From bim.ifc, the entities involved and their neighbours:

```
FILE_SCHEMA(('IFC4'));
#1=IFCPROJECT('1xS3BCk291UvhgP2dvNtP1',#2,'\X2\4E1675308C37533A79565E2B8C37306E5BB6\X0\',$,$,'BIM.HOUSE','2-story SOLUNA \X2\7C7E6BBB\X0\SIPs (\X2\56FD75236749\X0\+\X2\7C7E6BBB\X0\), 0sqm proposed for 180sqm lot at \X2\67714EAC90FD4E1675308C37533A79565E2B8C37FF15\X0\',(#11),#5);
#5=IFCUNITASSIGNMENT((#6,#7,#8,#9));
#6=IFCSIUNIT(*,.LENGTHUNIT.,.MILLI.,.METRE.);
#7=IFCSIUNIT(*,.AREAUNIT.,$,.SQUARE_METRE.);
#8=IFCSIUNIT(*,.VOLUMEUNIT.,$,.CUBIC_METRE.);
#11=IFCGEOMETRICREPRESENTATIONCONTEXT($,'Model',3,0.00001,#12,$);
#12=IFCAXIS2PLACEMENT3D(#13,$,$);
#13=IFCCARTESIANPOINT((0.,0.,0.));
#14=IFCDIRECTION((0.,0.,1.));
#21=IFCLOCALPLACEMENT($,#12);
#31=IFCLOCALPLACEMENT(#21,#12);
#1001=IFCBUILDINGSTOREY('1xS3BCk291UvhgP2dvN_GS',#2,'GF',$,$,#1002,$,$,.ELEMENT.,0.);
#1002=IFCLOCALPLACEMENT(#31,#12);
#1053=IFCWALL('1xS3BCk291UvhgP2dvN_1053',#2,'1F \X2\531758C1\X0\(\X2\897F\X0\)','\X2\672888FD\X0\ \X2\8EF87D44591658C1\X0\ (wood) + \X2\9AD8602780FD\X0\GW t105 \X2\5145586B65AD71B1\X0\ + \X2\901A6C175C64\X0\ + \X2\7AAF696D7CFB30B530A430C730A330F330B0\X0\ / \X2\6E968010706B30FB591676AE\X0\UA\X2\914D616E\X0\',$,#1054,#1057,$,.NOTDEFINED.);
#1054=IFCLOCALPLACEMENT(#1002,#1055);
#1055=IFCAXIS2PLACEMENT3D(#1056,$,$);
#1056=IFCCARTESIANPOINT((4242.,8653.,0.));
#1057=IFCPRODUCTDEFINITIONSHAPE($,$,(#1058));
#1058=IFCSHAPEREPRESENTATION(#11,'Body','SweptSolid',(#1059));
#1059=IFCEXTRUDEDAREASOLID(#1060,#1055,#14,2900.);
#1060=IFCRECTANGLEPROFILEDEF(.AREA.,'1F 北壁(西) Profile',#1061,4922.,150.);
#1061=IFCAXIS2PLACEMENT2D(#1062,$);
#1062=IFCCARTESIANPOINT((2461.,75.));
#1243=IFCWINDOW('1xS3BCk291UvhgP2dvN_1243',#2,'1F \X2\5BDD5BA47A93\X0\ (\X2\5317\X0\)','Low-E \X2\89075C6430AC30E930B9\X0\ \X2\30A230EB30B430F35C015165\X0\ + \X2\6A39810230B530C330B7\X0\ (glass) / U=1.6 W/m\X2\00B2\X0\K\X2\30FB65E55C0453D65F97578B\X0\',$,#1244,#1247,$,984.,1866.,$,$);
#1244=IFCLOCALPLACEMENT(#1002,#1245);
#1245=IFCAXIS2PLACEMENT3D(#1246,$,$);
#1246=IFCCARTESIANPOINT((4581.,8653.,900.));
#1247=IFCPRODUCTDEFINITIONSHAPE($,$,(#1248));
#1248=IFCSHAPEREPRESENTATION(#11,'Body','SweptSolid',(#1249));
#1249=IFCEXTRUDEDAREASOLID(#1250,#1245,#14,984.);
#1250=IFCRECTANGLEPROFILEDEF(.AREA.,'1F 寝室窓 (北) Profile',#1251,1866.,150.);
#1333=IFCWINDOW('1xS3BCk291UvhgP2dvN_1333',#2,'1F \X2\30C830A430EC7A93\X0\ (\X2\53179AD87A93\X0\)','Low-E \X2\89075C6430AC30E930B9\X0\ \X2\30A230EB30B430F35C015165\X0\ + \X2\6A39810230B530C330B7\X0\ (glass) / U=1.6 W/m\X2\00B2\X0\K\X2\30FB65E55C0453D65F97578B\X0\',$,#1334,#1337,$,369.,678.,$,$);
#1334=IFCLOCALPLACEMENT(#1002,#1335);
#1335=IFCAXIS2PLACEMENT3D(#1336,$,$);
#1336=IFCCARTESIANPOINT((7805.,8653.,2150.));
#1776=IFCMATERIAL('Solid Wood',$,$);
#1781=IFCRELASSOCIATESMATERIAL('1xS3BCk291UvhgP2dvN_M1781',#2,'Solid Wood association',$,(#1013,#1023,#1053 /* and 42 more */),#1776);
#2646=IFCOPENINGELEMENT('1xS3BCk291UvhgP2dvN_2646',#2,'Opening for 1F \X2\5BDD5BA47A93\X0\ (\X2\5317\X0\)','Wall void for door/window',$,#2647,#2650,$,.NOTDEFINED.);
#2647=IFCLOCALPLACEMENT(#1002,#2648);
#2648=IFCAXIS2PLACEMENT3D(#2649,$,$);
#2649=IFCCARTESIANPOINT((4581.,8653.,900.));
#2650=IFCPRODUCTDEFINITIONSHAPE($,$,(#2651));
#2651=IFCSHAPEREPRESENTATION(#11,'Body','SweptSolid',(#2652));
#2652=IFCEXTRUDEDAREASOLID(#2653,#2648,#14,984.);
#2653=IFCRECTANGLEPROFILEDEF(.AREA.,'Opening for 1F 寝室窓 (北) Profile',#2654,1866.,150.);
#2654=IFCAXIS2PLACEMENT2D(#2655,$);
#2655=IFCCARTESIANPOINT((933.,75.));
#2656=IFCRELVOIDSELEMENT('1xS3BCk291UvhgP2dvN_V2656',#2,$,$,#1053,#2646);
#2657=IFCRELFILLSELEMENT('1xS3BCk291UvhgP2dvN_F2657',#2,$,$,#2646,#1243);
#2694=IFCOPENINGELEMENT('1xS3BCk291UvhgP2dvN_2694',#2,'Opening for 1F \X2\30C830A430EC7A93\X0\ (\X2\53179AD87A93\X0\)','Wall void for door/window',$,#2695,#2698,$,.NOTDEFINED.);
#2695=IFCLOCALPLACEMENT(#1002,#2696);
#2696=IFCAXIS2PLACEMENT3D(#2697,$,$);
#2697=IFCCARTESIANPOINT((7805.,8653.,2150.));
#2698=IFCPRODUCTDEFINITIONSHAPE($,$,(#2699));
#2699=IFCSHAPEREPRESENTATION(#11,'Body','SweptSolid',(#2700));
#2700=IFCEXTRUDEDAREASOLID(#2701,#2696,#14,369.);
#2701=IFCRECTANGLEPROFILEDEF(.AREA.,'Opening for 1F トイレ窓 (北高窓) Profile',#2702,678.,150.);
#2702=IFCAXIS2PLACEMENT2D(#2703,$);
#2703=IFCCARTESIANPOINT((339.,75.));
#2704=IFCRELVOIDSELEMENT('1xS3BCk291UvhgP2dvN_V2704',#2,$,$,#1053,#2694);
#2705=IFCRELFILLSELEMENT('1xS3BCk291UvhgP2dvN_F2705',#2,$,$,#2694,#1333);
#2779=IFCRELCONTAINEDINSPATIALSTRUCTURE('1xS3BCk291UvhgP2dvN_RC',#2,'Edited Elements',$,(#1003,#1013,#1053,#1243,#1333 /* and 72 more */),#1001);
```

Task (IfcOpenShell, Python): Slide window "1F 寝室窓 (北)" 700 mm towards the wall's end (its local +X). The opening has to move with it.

```python
import ifcopenshell
import ifcopenshell.api.geometry
import ifcopenshell.util.placement
import ifcopenshell.util.unit

model = ifcopenshell.open("bim.ifc")
unit_scale = ifcopenshell.util.unit.calculate_unit_scale(model)

window = model.by_id(1243)
opening = window.FillsVoids[0].RelatingOpeningElement
wall = opening.VoidsElements[0].RelatingBuildingElement

wall_matrix = ifcopenshell.util.placement.get_local_placement(wall.ObjectPlacement)
shift = wall_matrix[:3, 0] * 0.7 / unit_scale
before = ifcopenshell.util.placement.get_local_placement(window.ObjectPlacement)[:3, 3].copy()

# The window is not placed relative to its opening, so move both.
for product in (opening, window):
    matrix = ifcopenshell.util.placement.get_local_placement(product.ObjectPlacement)
    matrix[:3, 3] += shift
    ifcopenshell.api.geometry.edit_object_placement(model, product=product, matrix=matrix, is_si=False)

after = ifcopenshell.util.placement.get_local_placement(window.ObjectPlacement)[:3, 3]
print("window moved by", (after - before).round(3) + 0.0)

model.write("bim-out.ifc")
```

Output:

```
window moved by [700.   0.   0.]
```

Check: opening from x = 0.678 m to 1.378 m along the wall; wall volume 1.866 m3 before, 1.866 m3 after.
